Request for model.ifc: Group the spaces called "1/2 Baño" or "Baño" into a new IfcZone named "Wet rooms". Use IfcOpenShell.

First a look at what the model holds.

```python
import ifcopenshell

model = ifcopenshell.open("model.ifc")
print(model.schema)
seen = {}
for space in model.by_type("IfcSpace"):
    seen[space.LongName] = seen.get(space.LongName, 0) + 1
for name, count in sorted(seen.items(), key=str):
    print(count, "x", name)
print("zones:", [z.Name for z in model.by_type("IfcZone")][:20])
```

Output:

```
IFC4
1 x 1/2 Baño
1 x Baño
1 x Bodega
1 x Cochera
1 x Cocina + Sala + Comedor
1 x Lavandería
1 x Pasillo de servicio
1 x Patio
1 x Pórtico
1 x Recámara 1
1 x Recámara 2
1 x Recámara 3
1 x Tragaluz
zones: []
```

```python
import ifcopenshell
import ifcopenshell.api.group
import ifcopenshell.api.root

model = ifcopenshell.open("model.ifc")

names = {"1/2 Baño", "Baño"}
spaces = [s for s in model.by_type("IfcSpace") if s.LongName in names]

zone = ifcopenshell.api.root.create_entity(model, ifc_class="IfcZone", name="Wet rooms")
ifcopenshell.api.group.assign_group(model, products=spaces, group=zone)
print(len(spaces), "spaces in", zone.Name)

model.write("model_updated.ifc")
```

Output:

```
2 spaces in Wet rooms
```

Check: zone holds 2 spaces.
